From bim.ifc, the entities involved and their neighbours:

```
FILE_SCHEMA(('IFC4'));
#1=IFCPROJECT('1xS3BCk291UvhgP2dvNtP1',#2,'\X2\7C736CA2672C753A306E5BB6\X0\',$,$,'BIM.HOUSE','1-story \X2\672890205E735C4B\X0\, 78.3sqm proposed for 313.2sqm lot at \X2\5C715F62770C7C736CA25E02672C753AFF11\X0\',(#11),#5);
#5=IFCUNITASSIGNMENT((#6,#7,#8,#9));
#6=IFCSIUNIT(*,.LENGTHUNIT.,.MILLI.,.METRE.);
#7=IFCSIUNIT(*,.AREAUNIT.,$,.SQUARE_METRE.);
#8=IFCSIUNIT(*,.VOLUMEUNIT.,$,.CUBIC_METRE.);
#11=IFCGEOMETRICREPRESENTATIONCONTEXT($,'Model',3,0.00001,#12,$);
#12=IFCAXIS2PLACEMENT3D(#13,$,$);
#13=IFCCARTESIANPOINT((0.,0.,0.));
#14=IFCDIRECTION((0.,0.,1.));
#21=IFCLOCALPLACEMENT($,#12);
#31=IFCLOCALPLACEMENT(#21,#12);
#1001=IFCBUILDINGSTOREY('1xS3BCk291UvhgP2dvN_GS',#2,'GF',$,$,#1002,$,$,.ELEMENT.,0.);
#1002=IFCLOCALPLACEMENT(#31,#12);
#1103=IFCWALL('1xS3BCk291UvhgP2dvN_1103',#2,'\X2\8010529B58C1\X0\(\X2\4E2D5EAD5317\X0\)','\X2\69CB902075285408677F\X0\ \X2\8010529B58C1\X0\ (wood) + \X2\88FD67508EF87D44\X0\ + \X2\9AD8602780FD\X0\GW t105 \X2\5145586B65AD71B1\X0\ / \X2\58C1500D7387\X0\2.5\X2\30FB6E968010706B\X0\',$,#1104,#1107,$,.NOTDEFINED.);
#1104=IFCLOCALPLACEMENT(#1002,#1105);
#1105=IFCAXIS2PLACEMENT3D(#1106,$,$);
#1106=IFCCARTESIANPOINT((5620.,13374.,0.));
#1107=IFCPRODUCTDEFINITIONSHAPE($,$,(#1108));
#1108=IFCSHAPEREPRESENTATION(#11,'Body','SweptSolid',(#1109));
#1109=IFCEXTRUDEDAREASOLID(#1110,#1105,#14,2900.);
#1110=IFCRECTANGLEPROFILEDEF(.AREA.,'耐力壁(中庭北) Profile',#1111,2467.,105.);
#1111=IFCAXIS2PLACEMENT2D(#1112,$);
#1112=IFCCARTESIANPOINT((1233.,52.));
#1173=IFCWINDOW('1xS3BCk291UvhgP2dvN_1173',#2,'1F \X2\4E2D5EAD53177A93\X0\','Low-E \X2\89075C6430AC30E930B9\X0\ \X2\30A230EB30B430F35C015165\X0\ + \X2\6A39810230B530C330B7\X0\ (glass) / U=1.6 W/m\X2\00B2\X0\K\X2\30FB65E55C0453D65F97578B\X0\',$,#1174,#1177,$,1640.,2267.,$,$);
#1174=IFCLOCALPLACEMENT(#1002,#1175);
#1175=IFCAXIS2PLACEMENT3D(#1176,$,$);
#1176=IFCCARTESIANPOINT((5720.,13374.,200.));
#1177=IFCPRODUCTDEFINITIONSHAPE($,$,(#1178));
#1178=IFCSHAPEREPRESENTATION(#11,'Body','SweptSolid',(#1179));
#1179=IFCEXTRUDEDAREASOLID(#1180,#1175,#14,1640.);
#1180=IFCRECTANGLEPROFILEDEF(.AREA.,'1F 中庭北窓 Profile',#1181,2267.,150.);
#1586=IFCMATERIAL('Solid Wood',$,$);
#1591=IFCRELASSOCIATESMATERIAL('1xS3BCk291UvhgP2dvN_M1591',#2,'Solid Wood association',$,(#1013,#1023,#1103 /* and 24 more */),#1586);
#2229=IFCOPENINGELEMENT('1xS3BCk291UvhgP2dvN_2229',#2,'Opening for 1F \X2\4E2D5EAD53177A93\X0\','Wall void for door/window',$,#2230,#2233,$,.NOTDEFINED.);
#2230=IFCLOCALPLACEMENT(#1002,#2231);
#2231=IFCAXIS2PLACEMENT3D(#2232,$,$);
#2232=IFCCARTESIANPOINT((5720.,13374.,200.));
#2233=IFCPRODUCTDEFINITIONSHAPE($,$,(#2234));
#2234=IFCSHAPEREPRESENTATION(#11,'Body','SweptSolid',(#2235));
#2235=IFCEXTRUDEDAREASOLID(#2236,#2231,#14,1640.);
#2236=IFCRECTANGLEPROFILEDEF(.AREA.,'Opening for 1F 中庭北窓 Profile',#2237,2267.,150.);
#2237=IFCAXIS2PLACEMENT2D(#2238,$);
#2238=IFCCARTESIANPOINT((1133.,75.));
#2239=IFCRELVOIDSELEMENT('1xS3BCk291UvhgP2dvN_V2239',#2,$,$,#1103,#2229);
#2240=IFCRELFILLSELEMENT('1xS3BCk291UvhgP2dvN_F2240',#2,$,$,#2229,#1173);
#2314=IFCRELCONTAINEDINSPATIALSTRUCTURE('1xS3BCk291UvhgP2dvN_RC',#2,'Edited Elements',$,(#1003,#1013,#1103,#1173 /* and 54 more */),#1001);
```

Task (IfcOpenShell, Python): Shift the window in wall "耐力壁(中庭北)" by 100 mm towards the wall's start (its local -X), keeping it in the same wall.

```python
import ifcopenshell
import ifcopenshell.api.geometry
import ifcopenshell.util.placement
import ifcopenshell.util.unit

model = ifcopenshell.open("bim.ifc")
unit_scale = ifcopenshell.util.unit.calculate_unit_scale(model)

window = model.by_guid("1xS3BCk291UvhgP2dvN_1173")
opening = window.FillsVoids[0].RelatingOpeningElement
wall = opening.VoidsElements[0].RelatingBuildingElement

wall_matrix = ifcopenshell.util.placement.get_local_placement(wall.ObjectPlacement)
shift = wall_matrix[:3, 0] * -0.1 / unit_scale
before = ifcopenshell.util.placement.get_local_placement(window.ObjectPlacement)[:3, 3].copy()

# The window is not placed relative to its opening, so move both.
for product in (opening, window):
    matrix = ifcopenshell.util.placement.get_local_placement(product.ObjectPlacement)
    matrix[:3, 3] += shift
    ifcopenshell.api.geometry.edit_object_placement(model, product=product, matrix=matrix, is_si=False)

after = ifcopenshell.util.placement.get_local_placement(window.ObjectPlacement)[:3, 3]
print("window moved by", (after - before).round(3) + 0.0)

model.write("bim_v2.ifc")
```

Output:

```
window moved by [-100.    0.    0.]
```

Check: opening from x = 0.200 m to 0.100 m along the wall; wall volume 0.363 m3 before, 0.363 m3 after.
